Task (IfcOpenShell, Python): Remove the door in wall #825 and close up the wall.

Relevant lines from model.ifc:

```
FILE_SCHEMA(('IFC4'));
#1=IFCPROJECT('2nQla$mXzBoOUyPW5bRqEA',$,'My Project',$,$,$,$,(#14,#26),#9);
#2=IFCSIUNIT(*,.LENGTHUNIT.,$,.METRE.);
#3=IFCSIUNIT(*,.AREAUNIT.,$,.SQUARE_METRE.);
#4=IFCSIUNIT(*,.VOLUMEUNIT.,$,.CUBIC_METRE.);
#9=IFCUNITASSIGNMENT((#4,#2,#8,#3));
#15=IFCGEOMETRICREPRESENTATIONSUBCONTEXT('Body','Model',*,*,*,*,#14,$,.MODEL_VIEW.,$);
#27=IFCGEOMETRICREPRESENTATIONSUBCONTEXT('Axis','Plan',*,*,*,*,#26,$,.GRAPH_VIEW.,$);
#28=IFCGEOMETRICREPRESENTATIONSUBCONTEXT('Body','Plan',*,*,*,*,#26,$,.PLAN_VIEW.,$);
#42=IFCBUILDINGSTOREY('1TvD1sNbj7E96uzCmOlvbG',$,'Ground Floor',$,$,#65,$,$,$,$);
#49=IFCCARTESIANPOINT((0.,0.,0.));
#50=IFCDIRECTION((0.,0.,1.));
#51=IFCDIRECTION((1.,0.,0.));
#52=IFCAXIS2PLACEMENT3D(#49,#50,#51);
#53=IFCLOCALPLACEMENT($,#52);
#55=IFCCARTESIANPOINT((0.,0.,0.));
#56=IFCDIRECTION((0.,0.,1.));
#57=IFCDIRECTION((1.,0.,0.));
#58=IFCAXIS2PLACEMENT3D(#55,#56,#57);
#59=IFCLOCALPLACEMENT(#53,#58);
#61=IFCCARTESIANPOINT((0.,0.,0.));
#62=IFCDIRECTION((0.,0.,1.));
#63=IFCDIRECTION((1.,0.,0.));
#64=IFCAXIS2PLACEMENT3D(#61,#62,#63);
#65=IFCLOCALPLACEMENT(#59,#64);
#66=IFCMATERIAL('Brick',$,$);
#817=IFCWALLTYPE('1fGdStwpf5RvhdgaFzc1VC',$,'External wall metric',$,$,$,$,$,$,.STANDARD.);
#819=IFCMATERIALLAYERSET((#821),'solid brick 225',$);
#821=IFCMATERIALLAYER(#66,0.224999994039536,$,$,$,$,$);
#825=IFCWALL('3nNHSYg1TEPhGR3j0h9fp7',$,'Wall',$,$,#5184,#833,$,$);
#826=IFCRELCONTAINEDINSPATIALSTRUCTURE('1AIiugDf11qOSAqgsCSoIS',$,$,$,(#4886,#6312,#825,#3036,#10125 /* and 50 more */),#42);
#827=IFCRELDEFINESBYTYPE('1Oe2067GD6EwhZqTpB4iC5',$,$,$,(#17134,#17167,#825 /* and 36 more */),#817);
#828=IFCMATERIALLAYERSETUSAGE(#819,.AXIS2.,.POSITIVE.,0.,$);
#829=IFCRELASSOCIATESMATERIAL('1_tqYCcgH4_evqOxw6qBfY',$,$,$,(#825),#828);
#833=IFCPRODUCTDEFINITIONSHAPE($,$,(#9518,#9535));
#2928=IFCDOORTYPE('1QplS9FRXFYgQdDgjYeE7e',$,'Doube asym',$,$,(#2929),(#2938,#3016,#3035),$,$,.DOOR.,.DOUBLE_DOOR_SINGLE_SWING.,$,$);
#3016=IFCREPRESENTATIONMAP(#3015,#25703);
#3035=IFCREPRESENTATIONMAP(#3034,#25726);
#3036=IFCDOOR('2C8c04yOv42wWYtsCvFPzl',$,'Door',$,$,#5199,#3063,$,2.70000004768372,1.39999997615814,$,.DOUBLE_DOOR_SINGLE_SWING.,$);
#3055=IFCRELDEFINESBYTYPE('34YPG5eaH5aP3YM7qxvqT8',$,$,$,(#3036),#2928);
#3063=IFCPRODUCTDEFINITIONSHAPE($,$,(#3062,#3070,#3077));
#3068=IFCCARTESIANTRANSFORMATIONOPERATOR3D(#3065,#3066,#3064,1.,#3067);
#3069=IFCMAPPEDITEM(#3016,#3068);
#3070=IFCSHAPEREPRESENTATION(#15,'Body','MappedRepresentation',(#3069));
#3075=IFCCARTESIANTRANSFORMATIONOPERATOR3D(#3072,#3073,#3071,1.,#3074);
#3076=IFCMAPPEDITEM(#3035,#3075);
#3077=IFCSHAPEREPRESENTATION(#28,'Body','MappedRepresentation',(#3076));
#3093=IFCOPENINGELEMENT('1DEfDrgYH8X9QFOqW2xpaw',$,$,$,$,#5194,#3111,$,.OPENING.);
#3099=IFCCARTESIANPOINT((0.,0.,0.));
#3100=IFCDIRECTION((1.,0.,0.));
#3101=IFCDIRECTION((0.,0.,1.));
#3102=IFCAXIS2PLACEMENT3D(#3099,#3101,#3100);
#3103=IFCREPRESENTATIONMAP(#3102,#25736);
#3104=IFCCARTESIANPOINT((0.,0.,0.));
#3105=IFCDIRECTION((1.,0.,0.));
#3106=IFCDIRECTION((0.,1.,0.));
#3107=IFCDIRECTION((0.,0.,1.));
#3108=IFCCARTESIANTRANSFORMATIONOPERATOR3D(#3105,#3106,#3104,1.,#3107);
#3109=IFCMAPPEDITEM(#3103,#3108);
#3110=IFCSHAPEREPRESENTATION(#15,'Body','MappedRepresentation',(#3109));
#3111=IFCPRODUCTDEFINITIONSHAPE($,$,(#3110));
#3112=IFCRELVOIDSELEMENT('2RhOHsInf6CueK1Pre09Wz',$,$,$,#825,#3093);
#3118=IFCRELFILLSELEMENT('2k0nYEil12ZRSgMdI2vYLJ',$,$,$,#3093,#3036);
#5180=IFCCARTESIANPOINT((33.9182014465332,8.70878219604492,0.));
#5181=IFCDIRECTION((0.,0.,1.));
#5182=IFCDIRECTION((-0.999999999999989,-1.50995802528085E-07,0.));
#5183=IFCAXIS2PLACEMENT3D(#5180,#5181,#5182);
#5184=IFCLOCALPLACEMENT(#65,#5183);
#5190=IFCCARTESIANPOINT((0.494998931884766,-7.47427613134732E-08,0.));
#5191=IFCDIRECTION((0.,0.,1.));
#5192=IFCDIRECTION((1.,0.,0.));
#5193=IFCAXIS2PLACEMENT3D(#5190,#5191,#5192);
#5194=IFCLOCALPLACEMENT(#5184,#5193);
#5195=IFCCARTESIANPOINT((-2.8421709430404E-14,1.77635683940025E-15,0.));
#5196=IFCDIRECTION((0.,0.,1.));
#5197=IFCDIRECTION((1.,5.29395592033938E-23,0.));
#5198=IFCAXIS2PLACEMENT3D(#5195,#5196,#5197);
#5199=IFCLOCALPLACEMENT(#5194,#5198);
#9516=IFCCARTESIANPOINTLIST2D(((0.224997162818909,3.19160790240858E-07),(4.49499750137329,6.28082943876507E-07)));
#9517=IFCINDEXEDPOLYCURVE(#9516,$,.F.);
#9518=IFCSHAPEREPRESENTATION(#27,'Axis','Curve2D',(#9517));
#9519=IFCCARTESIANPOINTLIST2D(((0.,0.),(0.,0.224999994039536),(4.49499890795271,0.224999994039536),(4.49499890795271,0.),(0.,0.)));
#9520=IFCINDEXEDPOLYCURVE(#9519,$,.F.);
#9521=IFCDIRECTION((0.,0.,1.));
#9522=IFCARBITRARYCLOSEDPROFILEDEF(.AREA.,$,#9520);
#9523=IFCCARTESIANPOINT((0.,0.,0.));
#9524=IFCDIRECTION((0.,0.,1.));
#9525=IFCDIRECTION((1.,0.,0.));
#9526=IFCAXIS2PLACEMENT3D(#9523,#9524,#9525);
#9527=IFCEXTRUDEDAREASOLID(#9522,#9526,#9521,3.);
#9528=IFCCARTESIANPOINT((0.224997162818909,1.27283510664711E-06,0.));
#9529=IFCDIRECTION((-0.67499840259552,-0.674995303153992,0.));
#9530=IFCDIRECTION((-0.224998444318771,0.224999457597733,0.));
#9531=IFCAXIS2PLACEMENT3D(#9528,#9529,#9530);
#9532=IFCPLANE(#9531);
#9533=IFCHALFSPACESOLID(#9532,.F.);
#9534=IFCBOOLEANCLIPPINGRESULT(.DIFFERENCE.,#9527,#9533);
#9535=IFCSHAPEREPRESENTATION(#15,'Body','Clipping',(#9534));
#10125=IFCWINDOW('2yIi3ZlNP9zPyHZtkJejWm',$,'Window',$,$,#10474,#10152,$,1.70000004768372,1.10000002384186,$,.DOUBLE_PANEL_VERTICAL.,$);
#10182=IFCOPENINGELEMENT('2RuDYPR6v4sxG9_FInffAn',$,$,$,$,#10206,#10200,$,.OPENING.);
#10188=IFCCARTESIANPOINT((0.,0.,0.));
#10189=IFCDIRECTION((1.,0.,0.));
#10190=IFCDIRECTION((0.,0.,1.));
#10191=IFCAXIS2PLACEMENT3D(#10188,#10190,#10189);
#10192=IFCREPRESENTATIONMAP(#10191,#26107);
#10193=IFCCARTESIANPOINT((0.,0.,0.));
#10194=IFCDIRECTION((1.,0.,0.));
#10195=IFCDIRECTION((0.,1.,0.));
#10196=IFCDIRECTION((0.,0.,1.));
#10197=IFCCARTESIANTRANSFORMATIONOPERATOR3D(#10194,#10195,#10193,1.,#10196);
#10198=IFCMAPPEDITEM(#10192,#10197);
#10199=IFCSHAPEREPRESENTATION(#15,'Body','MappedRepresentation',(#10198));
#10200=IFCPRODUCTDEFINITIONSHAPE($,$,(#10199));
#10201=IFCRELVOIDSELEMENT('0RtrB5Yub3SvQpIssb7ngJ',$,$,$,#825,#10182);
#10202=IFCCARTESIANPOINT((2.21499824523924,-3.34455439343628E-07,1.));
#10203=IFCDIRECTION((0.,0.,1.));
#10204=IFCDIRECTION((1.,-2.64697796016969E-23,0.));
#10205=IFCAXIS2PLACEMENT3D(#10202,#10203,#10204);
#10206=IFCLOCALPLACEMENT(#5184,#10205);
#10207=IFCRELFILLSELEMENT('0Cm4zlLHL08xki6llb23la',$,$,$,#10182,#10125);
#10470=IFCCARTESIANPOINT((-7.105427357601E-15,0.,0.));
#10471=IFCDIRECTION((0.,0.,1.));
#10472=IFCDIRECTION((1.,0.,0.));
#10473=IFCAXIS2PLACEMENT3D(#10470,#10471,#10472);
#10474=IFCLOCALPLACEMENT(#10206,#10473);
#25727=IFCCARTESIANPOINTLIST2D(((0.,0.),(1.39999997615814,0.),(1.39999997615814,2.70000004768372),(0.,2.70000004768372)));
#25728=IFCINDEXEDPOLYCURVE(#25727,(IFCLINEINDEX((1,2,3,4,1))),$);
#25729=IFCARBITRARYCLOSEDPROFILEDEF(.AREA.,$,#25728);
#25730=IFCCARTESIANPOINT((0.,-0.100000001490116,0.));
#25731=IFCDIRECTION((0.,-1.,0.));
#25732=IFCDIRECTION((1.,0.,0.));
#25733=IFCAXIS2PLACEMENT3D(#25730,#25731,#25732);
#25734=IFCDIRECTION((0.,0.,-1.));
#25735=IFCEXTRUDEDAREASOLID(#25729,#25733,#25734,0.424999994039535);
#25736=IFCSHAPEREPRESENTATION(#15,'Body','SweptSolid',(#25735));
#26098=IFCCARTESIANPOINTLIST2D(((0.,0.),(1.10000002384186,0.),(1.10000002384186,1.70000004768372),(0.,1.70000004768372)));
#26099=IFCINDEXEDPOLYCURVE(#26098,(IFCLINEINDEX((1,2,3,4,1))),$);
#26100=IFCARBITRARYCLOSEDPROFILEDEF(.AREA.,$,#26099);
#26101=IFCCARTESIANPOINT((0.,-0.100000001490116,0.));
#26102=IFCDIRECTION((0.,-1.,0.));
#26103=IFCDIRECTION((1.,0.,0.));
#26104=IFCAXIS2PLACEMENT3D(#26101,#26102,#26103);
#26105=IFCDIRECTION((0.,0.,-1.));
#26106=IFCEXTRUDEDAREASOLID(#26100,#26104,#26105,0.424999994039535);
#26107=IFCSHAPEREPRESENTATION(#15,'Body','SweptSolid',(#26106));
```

```python
import ifcopenshell
import ifcopenshell.api.feature
import ifcopenshell.api.root
import ifcopenshell.geom
import ifcopenshell.util.shape

model = ifcopenshell.open("model.ifc")
settings = ifcopenshell.geom.settings()


def volume(element):
    """Net volume in cubic metres, openings subtracted."""
    shape = ifcopenshell.geom.create_shape(settings, element)
    return ifcopenshell.util.shape.get_volume(shape.geometry)


door = model.by_guid("2C8c04yOv42wWYtsCvFPzl")
opening = door.FillsVoids[0].RelatingOpeningElement
wall = opening.VoidsElements[0].RelatingBuildingElement
before = volume(wall)

ifcopenshell.api.root.remove_product(model, product=door)
ifcopenshell.api.feature.remove_feature(model, feature=opening)

after = volume(wall)

print(f"wall volume {before:.3f} -> {after:.3f} m3")

model.write("model-out.ifc")
```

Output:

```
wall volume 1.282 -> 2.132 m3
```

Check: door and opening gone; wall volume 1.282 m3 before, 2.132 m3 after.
